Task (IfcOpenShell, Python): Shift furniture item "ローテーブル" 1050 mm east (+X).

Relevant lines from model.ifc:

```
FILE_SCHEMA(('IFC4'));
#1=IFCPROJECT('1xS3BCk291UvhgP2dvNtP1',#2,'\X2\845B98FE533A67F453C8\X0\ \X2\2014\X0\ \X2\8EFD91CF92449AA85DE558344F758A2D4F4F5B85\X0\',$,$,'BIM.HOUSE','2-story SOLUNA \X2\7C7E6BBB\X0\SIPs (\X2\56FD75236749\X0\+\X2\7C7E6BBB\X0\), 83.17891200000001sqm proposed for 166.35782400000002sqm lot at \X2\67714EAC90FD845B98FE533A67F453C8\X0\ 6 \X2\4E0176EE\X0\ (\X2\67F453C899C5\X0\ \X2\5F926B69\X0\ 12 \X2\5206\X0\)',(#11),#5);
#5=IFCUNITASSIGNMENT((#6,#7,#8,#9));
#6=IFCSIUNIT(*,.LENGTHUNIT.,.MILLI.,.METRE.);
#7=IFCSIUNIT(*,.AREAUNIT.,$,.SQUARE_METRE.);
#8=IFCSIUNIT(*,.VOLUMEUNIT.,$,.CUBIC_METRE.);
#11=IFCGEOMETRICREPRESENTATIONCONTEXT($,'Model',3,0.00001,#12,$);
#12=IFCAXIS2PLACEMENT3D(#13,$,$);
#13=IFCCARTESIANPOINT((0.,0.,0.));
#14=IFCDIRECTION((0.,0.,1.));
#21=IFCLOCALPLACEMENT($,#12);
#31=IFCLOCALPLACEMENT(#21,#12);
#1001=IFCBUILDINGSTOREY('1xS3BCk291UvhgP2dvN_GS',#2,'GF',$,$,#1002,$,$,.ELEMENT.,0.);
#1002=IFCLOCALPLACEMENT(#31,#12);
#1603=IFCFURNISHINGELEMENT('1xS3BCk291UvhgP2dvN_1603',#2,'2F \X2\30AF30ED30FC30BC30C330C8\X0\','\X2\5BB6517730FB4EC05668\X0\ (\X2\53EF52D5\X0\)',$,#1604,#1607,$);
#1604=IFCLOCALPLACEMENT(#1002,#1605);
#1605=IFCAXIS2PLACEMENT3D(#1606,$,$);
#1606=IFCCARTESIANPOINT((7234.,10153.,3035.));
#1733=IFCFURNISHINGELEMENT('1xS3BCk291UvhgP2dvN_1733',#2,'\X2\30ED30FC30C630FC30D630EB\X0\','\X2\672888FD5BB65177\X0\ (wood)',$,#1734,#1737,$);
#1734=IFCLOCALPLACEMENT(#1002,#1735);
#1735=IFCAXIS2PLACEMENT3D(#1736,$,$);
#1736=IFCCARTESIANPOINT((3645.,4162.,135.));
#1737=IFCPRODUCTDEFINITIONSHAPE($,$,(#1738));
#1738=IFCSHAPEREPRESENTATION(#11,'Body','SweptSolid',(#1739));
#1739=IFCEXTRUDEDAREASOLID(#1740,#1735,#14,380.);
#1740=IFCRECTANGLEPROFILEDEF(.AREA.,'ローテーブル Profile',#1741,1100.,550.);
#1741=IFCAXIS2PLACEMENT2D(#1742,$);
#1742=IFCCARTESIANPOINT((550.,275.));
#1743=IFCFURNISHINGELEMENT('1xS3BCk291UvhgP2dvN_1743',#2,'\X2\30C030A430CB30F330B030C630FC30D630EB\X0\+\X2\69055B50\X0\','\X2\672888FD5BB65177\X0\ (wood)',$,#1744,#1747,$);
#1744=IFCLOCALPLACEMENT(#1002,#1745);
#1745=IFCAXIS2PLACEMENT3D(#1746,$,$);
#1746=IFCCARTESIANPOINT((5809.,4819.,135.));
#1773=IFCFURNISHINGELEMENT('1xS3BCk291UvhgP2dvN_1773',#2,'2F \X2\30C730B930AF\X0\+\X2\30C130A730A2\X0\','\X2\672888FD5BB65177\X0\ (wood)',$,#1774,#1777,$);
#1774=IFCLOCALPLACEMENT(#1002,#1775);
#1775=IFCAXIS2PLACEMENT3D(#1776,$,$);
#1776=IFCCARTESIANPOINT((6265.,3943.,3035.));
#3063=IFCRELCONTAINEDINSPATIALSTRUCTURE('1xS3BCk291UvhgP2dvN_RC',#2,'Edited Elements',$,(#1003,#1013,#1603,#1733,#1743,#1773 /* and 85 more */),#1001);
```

```python
import ifcopenshell
import ifcopenshell.api.geometry
import ifcopenshell.util.placement
import ifcopenshell.util.unit

model = ifcopenshell.open("model.ifc")
unit_scale = ifcopenshell.util.unit.calculate_unit_scale(model)

item = model.by_guid("1xS3BCk291UvhgP2dvN_1733")
matrix = ifcopenshell.util.placement.get_local_placement(item.ObjectPlacement)
matrix[0, 3] += 1.05 / unit_scale
ifcopenshell.api.geometry.edit_object_placement(model, product=item, matrix=matrix, is_si=False)

print(ifcopenshell.util.placement.get_local_placement(item.ObjectPlacement).round(3) + 0.0)

model.write("model-out.ifc")
```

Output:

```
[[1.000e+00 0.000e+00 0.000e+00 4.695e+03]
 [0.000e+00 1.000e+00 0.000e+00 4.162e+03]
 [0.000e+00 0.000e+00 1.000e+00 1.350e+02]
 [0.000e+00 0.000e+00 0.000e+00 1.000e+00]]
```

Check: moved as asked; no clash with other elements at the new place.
